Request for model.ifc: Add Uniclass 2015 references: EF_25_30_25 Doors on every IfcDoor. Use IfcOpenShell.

First a look at what the model holds.

```python
import ifcopenshell

model = ifcopenshell.open("model.ifc")
print(model.schema)
print("classifications:", [c.Name for c in model.by_type("IfcClassification")])
for ifc_class in ("IfcDoor", "IfcRoof", "IfcStair", "IfcWall", "IfcWindow"):
    print(ifc_class, len(model.by_type(ifc_class)))
```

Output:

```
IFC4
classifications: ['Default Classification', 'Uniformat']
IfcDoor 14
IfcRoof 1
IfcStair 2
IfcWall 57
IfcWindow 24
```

```python
import ifcopenshell
import ifcopenshell.api.classification

model = ifcopenshell.open("model.ifc")

system = ifcopenshell.api.classification.add_classification(model, classification="Uniclass 2015")

codes = {
    "IfcDoor": ("EF_25_30_25", "Doors"),
}
for ifc_class, (code, name) in codes.items():
    products = model.by_type(ifc_class)
    ifcopenshell.api.classification.add_reference(
        model, products=products, classification=system, identification=code, name=name
    )
    print(code, len(products))

model.write("model_rev.ifc")
```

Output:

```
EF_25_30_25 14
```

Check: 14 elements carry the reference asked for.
